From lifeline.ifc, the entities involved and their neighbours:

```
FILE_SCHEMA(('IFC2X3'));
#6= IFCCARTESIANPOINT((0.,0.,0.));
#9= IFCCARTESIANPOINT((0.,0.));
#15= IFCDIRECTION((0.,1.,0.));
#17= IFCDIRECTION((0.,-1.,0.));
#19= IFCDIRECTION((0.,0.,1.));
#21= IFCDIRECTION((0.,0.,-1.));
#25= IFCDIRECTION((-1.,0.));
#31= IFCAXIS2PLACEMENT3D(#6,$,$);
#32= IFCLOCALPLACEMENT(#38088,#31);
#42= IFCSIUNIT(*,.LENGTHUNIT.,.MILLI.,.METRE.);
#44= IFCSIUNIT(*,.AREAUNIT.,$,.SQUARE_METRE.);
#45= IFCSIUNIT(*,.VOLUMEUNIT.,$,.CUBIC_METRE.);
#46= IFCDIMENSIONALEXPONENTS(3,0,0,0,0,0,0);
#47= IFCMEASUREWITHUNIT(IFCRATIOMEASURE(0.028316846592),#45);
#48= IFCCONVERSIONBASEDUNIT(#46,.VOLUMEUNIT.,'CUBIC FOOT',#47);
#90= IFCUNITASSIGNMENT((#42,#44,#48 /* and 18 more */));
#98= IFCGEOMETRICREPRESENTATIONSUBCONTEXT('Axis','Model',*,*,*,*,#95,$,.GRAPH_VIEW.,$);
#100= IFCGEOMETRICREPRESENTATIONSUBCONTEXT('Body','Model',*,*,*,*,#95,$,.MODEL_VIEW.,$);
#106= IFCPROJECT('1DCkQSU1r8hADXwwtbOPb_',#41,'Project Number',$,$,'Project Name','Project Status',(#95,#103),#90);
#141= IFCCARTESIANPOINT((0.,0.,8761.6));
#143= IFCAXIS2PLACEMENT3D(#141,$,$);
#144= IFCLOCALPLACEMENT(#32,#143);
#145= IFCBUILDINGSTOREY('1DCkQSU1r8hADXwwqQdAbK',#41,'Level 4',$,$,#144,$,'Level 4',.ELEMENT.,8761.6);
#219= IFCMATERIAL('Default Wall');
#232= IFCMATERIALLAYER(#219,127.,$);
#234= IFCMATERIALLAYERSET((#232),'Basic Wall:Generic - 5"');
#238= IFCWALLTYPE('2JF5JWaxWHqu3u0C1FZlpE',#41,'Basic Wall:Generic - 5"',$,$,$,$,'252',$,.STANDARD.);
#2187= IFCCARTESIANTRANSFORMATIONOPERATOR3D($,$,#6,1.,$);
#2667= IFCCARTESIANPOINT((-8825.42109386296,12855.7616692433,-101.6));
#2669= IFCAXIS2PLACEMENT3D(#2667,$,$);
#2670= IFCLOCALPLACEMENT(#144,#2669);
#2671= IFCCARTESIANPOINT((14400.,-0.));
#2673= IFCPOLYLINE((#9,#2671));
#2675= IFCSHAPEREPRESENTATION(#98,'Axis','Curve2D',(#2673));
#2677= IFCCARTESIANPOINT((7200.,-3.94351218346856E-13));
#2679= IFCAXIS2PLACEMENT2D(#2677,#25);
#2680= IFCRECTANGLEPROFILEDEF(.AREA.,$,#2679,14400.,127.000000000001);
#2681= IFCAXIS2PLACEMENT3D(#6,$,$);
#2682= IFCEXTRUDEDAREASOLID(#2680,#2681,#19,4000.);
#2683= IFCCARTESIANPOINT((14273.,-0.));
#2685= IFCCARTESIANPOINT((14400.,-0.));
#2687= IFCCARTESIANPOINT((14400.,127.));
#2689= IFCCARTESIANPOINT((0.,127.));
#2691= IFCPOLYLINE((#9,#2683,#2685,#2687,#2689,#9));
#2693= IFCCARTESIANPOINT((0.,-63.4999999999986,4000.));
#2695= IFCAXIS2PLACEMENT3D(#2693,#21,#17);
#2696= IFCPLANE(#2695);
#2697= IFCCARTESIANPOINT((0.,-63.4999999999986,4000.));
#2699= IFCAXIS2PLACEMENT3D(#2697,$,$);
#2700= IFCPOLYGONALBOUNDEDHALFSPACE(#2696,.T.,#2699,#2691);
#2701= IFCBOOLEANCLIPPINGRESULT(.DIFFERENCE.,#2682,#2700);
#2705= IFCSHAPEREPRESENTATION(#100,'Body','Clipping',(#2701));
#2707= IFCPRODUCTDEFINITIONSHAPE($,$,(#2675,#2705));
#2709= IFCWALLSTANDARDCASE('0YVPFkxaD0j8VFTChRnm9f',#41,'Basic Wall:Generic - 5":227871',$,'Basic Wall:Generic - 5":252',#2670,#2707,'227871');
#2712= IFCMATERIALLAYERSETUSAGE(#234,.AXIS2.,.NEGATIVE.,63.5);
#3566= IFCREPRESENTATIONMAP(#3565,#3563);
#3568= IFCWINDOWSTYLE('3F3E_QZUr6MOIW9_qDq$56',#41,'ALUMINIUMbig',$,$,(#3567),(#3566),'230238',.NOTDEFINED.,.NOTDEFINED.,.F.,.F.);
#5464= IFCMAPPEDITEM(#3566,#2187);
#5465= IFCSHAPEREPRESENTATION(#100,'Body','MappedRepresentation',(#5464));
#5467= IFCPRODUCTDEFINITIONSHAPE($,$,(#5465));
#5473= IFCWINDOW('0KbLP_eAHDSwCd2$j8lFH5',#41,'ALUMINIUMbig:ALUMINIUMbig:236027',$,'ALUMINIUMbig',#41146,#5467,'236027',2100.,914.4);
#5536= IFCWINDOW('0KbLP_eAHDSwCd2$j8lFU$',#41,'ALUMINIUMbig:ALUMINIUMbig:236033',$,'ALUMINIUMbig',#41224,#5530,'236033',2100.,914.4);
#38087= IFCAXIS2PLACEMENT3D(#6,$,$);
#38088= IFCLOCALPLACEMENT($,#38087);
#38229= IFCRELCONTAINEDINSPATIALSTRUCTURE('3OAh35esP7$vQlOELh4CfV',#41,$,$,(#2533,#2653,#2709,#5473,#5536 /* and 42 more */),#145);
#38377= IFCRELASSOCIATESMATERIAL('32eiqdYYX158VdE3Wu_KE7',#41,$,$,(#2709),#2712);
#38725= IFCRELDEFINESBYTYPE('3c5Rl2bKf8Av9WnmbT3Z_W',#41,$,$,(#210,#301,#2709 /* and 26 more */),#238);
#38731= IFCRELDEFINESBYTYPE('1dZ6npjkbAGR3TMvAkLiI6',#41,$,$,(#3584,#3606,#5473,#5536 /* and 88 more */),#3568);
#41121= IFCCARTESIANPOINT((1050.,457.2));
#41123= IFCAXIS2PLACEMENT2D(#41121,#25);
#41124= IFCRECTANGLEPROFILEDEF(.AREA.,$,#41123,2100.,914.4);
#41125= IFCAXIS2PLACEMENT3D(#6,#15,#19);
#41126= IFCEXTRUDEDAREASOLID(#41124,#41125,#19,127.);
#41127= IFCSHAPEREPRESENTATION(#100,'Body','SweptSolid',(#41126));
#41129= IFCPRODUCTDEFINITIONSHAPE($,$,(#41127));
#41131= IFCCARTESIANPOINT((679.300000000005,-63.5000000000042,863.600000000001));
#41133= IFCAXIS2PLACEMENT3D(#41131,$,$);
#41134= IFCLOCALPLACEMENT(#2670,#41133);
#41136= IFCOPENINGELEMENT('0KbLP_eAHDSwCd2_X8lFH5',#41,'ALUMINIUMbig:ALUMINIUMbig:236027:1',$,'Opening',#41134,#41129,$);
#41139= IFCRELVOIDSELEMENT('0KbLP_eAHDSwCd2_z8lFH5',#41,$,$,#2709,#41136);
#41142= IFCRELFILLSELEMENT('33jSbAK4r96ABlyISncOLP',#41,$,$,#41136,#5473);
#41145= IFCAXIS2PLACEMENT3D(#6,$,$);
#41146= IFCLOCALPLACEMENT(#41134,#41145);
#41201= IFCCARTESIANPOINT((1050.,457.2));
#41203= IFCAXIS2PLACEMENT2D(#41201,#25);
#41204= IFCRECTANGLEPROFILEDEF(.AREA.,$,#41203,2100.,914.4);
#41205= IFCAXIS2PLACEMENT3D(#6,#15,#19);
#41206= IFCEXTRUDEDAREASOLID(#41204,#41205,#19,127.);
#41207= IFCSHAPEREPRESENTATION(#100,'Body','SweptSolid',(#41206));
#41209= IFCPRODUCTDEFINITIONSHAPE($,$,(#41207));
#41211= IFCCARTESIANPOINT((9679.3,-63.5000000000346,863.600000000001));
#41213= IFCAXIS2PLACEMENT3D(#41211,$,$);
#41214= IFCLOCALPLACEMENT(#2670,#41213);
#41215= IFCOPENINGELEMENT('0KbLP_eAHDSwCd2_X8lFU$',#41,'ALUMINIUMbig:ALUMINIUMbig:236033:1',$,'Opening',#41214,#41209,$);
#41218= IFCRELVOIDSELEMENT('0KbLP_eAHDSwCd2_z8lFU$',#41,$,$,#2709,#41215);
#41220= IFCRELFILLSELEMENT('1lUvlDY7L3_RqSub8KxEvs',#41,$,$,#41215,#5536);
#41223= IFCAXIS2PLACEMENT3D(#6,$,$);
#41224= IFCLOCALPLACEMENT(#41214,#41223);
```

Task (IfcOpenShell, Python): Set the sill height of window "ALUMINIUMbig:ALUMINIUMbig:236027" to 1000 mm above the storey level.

```python
import numpy as np
import ifcopenshell
import ifcopenshell.api.geometry
import ifcopenshell.geom
import ifcopenshell.util.element
import ifcopenshell.util.placement
import ifcopenshell.util.shape
import ifcopenshell.util.unit

model = ifcopenshell.open("lifeline.ifc")
unit_scale = ifcopenshell.util.unit.calculate_unit_scale(model)

window = model.by_guid("0KbLP_eAHDSwCd2$j8lFH5")
opening = window.FillsVoids[0].RelatingOpeningElement
storey = ifcopenshell.util.element.get_container(window, ifc_class="IfcBuildingStorey")
level = ifcopenshell.util.placement.get_local_placement(storey.ObjectPlacement)[2, 3]

# The opening's origin need not be at the sill, so measure its lowest point.
shape = ifcopenshell.geom.create_shape(ifcopenshell.geom.settings(), opening)
bottom = ifcopenshell.util.shape.get_shape_bottom_elevation(shape, shape.geometry) / unit_scale
dz = level + 1 / unit_scale - bottom

shift = np.array([0.0, 0.0, dz])
# The window is placed relative to its opening, so it follows when the opening moves.
matrix = ifcopenshell.util.placement.get_local_placement(opening.ObjectPlacement)
matrix[:3, 3] += shift
ifcopenshell.api.geometry.edit_object_placement(
    model, product=opening, matrix=matrix, is_si=False, should_transform_children=True
)

print(f"moved by {dz * unit_scale:+.3f} m")

model.write("lifeline-out.ifc")
```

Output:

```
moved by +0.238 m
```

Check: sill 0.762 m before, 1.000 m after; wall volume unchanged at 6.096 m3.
